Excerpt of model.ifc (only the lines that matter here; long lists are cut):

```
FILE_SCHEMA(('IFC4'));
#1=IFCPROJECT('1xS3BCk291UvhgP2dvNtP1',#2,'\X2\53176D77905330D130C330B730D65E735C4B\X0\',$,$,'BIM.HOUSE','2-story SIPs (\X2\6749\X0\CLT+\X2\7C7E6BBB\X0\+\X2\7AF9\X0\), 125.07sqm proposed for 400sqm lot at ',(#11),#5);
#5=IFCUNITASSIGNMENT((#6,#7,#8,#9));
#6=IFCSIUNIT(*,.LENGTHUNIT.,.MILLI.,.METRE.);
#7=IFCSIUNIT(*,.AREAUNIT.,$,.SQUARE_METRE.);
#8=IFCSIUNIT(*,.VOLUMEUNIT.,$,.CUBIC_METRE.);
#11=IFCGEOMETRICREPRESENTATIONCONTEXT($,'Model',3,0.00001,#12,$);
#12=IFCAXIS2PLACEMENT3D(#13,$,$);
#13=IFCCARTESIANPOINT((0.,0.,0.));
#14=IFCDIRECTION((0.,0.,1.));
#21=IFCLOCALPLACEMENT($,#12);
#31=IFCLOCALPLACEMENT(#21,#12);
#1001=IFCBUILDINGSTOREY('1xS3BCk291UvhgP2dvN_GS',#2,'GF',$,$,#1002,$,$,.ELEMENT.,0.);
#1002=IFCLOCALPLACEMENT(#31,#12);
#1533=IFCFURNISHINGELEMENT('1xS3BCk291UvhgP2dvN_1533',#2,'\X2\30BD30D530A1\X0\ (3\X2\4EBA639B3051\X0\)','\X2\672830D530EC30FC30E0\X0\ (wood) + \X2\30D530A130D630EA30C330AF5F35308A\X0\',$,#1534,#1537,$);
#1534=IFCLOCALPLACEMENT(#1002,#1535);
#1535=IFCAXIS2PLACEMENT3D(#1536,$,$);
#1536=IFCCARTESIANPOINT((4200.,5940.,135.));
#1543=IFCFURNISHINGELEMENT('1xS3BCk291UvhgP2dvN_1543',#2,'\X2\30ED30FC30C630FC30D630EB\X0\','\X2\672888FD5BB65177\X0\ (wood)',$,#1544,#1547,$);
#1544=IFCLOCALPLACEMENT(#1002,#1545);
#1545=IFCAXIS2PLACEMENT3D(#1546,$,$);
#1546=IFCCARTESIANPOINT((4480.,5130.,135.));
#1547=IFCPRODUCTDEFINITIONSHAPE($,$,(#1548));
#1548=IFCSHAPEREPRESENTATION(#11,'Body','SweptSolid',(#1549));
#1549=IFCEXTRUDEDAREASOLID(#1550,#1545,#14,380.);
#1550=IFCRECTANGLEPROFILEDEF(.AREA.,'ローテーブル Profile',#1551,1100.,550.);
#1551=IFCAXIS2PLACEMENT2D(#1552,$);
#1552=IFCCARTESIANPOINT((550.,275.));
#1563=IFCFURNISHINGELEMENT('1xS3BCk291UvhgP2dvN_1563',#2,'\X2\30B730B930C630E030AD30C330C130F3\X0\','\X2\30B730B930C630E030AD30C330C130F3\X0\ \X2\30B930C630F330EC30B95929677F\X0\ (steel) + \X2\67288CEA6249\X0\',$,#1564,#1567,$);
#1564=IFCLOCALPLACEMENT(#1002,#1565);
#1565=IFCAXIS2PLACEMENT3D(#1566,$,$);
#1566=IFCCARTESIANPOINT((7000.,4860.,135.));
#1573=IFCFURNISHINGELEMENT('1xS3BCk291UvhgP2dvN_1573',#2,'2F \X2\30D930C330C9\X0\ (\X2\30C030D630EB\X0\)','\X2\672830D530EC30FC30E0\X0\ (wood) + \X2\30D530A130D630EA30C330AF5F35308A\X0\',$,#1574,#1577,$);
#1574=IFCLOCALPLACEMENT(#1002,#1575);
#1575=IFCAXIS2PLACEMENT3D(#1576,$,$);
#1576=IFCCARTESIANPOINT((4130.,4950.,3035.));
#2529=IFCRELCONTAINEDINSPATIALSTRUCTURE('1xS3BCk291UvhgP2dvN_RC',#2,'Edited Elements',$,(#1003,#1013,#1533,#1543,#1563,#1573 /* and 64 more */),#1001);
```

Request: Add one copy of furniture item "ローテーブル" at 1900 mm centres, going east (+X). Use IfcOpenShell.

```python
import numpy as np
import ifcopenshell
import ifcopenshell.api.geometry
import ifcopenshell.api.root
import ifcopenshell.util.element
import ifcopenshell.util.placement

model = ifcopenshell.open("model.ifc")


def reuse_history(source, copy):
    """copy_class also copies each property set's owner history, people and application; keep the originals."""
    for rel in copy.IsDefinedBy:
        if rel.is_a("IfcRelDefinesByProperties") and (history := rel.RelatingPropertyDefinition.OwnerHistory):
            rel.RelatingPropertyDefinition.OwnerHistory = source.OwnerHistory
            ifcopenshell.util.element.remove_deep2(model, history)


source = model.by_guid("1xS3BCk291UvhgP2dvN_1543")
base = ifcopenshell.util.placement.get_local_placement(source.ObjectPlacement)
step = np.array([1.0, 0.0, 0.0]) * 1900.0

for i in range(1, 2):
    copy = ifcopenshell.api.root.copy_class(model, product=source)
    copy.Representation = ifcopenshell.util.element.copy_deep(
        model, source.Representation, exclude=["IfcGeometricRepresentationContext", "IfcRepresentationMap"]
    )
    reuse_history(source, copy)
    matrix = base.copy()
    matrix[:3, 3] += i * step
    print("added at", matrix[:3, 3].round(3) + 0.0)
    ifcopenshell.api.geometry.edit_object_placement(model, product=copy, matrix=matrix, is_si=False)

model.write("model-out.ifc")
```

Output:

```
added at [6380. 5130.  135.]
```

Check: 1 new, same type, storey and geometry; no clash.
